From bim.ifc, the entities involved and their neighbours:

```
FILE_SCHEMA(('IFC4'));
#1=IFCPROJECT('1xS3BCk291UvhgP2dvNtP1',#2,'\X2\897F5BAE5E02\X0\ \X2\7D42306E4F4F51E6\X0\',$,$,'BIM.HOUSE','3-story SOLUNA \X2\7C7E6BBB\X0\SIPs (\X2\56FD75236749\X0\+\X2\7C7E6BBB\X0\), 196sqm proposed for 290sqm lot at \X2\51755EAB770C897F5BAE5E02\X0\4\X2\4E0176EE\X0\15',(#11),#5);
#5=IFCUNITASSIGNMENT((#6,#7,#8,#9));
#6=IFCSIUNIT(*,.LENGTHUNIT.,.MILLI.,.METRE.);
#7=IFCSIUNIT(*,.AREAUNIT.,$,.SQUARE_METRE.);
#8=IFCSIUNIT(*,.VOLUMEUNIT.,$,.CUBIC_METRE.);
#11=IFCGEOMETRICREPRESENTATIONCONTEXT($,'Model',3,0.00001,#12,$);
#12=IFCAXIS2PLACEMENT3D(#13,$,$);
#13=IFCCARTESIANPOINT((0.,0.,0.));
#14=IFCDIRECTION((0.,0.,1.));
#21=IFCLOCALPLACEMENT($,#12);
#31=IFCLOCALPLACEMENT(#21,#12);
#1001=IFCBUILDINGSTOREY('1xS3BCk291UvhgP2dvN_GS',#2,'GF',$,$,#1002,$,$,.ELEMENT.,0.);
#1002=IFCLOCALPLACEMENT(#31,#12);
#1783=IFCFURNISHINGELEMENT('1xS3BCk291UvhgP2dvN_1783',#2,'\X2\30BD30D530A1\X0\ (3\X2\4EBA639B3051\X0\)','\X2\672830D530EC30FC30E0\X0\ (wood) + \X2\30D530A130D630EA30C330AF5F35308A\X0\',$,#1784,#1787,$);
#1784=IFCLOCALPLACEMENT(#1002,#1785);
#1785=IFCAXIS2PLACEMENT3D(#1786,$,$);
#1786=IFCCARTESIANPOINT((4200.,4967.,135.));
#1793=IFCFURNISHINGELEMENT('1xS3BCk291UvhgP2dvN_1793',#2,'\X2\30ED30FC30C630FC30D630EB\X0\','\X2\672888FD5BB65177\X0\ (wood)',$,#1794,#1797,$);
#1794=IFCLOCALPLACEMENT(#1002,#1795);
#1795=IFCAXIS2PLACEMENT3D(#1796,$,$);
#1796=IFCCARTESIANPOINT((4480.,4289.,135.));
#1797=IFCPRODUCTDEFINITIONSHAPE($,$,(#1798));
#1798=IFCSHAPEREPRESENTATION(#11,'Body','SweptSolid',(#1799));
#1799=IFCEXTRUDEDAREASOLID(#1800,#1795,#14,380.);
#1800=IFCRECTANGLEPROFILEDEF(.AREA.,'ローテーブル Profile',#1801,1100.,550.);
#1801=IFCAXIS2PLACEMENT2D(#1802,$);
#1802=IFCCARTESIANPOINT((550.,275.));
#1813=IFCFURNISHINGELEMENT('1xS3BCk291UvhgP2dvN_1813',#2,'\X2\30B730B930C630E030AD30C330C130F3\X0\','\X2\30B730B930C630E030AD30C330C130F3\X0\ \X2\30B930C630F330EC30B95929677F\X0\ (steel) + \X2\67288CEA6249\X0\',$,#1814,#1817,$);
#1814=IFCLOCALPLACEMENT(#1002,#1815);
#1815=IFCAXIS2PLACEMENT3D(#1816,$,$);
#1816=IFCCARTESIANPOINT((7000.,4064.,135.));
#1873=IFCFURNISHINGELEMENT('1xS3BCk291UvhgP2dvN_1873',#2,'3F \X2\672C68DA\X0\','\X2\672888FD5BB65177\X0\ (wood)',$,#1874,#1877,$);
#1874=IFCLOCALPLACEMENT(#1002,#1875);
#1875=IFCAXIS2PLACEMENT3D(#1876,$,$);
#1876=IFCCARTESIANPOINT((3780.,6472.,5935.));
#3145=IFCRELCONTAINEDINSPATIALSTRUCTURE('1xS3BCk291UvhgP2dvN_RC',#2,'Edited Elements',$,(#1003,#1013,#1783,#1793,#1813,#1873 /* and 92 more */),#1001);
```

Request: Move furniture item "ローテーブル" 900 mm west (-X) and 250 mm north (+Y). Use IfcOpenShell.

```python
import ifcopenshell
import ifcopenshell.api.geometry
import ifcopenshell.util.placement
import ifcopenshell.util.unit

model = ifcopenshell.open("bim.ifc")
unit_scale = ifcopenshell.util.unit.calculate_unit_scale(model)

item = model.by_guid("1xS3BCk291UvhgP2dvN_1793")
matrix = ifcopenshell.util.placement.get_local_placement(item.ObjectPlacement)
matrix[0, 3] -= 0.9 / unit_scale
matrix[1, 3] += 0.25 / unit_scale
ifcopenshell.api.geometry.edit_object_placement(model, product=item, matrix=matrix, is_si=False)

print(ifcopenshell.util.placement.get_local_placement(item.ObjectPlacement).round(3) + 0.0)

model.write("bim_edited.ifc")
```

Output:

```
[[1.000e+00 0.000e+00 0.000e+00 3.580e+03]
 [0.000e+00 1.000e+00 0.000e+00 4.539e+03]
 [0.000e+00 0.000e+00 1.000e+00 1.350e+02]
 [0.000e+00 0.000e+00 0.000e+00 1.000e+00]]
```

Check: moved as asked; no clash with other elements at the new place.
